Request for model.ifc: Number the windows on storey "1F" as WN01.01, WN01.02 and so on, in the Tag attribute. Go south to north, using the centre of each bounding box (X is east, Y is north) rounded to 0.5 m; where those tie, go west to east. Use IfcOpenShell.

First a look at what the model holds.

```python
import ifcopenshell
import ifcopenshell.util.element
import ifcopenshell.util.placement

model = ifcopenshell.open("model.ifc")
print(model.schema)
storey = next(s for s in model.by_type("IfcBuildingStorey") if s.Name == "1F")
windows = [e for e in ifcopenshell.util.element.get_decomposition(storey) if e.is_a("IfcWindow")]
for e in sorted(windows, key=lambda e: e.id()):
    origin = ifcopenshell.util.placement.get_local_placement(e.ObjectPlacement)[:3, 3]
    print(e.id(), e.Tag, e.Name, origin.round(2) + 0.0, sep=" | ")
```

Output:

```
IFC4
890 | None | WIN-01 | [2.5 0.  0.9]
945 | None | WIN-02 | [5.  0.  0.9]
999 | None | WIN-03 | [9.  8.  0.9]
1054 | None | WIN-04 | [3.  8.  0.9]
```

```python
import ifcopenshell
import ifcopenshell.geom
import ifcopenshell.util.element
import ifcopenshell.util.shape

model = ifcopenshell.open("model.ifc")
settings = ifcopenshell.geom.settings()
settings.set("use-world-coords", True)


def centre(element):
    shape = ifcopenshell.geom.create_shape(settings, element)
    return ifcopenshell.util.shape.get_bbox_centroid(shape.geometry)


storey = next(s for s in model.by_type("IfcBuildingStorey") if s.Name == "1F")
windows = [e for e in ifcopenshell.util.element.get_decomposition(storey) if e.is_a("IfcWindow")]

# Insertion points can sit at a corner or the storey origin, so sort by the geometry (in metres).
centres = {e: centre(e) for e in windows}
windows.sort(key=lambda e: (round(centres[e][1] / 0.5), centres[e][0]))

for i, e in enumerate(windows, start=1):
    number = f"WN01.{i:02d}"
    e.Tag = number
    print(e.id(), number)

model.write("model-out.ifc")
```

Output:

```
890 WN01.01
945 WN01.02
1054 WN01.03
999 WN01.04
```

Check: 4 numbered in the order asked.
